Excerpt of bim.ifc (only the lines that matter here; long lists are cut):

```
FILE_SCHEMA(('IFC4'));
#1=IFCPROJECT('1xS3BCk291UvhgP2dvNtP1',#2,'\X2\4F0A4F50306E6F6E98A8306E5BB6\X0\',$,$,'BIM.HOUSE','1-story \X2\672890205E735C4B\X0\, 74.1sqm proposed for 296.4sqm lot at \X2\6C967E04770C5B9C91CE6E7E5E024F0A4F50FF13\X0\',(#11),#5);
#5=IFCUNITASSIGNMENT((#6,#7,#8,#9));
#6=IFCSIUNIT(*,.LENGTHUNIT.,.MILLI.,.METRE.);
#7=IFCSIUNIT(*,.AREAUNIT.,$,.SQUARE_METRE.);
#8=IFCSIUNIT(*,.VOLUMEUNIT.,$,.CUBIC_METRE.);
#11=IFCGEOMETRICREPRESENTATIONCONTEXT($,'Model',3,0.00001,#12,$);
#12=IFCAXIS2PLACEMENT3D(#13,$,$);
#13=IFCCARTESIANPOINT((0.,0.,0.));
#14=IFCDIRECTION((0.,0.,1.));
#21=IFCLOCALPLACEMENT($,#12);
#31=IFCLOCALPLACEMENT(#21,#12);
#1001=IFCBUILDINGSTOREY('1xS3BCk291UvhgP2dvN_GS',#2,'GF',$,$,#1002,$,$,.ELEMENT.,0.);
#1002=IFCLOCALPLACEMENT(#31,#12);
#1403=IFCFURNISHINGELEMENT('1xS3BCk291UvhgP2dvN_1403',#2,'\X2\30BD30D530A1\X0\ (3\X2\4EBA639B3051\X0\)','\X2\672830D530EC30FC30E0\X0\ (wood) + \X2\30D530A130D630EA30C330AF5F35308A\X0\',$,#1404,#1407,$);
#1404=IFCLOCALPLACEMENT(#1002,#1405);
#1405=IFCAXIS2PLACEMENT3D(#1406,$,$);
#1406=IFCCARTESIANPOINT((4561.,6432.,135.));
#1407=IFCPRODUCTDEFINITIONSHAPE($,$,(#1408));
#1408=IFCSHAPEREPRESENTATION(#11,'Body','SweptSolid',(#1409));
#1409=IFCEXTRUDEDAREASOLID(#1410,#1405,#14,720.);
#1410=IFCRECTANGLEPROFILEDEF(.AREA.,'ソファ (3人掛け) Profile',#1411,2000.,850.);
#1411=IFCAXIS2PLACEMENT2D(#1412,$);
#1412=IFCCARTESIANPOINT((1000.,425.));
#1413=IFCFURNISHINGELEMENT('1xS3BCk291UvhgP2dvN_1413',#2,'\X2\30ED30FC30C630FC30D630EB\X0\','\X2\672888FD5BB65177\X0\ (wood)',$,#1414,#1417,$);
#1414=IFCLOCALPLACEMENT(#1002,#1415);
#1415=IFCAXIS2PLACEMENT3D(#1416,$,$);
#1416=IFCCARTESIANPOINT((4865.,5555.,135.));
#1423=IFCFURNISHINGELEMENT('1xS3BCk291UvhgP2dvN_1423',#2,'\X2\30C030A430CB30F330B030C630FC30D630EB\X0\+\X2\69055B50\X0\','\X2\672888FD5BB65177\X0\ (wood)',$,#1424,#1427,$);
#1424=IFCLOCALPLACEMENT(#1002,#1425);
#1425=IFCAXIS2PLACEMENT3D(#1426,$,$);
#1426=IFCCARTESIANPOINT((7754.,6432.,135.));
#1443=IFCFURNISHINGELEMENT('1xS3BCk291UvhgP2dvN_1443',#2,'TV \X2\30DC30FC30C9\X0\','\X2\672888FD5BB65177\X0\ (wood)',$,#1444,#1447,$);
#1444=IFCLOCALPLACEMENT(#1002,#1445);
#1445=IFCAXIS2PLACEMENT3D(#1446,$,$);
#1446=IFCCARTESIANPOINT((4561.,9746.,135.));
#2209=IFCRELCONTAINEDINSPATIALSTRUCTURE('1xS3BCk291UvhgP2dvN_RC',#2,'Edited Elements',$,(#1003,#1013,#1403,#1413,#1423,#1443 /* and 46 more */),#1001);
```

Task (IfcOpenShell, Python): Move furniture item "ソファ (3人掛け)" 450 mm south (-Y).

```python
import ifcopenshell
import ifcopenshell.api.geometry
import ifcopenshell.util.placement
import ifcopenshell.util.unit

model = ifcopenshell.open("bim.ifc")
unit_scale = ifcopenshell.util.unit.calculate_unit_scale(model)

item = model.by_id(1403)
matrix = ifcopenshell.util.placement.get_local_placement(item.ObjectPlacement)
matrix[1, 3] -= 0.45 / unit_scale
ifcopenshell.api.geometry.edit_object_placement(model, product=item, matrix=matrix, is_si=False)

print(ifcopenshell.util.placement.get_local_placement(item.ObjectPlacement).round(3) + 0.0)

model.write("bim-out.ifc")
```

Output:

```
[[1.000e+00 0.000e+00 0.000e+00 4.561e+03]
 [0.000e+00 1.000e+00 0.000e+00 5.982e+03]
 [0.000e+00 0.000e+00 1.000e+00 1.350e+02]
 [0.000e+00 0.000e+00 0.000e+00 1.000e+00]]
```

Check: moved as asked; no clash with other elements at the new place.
